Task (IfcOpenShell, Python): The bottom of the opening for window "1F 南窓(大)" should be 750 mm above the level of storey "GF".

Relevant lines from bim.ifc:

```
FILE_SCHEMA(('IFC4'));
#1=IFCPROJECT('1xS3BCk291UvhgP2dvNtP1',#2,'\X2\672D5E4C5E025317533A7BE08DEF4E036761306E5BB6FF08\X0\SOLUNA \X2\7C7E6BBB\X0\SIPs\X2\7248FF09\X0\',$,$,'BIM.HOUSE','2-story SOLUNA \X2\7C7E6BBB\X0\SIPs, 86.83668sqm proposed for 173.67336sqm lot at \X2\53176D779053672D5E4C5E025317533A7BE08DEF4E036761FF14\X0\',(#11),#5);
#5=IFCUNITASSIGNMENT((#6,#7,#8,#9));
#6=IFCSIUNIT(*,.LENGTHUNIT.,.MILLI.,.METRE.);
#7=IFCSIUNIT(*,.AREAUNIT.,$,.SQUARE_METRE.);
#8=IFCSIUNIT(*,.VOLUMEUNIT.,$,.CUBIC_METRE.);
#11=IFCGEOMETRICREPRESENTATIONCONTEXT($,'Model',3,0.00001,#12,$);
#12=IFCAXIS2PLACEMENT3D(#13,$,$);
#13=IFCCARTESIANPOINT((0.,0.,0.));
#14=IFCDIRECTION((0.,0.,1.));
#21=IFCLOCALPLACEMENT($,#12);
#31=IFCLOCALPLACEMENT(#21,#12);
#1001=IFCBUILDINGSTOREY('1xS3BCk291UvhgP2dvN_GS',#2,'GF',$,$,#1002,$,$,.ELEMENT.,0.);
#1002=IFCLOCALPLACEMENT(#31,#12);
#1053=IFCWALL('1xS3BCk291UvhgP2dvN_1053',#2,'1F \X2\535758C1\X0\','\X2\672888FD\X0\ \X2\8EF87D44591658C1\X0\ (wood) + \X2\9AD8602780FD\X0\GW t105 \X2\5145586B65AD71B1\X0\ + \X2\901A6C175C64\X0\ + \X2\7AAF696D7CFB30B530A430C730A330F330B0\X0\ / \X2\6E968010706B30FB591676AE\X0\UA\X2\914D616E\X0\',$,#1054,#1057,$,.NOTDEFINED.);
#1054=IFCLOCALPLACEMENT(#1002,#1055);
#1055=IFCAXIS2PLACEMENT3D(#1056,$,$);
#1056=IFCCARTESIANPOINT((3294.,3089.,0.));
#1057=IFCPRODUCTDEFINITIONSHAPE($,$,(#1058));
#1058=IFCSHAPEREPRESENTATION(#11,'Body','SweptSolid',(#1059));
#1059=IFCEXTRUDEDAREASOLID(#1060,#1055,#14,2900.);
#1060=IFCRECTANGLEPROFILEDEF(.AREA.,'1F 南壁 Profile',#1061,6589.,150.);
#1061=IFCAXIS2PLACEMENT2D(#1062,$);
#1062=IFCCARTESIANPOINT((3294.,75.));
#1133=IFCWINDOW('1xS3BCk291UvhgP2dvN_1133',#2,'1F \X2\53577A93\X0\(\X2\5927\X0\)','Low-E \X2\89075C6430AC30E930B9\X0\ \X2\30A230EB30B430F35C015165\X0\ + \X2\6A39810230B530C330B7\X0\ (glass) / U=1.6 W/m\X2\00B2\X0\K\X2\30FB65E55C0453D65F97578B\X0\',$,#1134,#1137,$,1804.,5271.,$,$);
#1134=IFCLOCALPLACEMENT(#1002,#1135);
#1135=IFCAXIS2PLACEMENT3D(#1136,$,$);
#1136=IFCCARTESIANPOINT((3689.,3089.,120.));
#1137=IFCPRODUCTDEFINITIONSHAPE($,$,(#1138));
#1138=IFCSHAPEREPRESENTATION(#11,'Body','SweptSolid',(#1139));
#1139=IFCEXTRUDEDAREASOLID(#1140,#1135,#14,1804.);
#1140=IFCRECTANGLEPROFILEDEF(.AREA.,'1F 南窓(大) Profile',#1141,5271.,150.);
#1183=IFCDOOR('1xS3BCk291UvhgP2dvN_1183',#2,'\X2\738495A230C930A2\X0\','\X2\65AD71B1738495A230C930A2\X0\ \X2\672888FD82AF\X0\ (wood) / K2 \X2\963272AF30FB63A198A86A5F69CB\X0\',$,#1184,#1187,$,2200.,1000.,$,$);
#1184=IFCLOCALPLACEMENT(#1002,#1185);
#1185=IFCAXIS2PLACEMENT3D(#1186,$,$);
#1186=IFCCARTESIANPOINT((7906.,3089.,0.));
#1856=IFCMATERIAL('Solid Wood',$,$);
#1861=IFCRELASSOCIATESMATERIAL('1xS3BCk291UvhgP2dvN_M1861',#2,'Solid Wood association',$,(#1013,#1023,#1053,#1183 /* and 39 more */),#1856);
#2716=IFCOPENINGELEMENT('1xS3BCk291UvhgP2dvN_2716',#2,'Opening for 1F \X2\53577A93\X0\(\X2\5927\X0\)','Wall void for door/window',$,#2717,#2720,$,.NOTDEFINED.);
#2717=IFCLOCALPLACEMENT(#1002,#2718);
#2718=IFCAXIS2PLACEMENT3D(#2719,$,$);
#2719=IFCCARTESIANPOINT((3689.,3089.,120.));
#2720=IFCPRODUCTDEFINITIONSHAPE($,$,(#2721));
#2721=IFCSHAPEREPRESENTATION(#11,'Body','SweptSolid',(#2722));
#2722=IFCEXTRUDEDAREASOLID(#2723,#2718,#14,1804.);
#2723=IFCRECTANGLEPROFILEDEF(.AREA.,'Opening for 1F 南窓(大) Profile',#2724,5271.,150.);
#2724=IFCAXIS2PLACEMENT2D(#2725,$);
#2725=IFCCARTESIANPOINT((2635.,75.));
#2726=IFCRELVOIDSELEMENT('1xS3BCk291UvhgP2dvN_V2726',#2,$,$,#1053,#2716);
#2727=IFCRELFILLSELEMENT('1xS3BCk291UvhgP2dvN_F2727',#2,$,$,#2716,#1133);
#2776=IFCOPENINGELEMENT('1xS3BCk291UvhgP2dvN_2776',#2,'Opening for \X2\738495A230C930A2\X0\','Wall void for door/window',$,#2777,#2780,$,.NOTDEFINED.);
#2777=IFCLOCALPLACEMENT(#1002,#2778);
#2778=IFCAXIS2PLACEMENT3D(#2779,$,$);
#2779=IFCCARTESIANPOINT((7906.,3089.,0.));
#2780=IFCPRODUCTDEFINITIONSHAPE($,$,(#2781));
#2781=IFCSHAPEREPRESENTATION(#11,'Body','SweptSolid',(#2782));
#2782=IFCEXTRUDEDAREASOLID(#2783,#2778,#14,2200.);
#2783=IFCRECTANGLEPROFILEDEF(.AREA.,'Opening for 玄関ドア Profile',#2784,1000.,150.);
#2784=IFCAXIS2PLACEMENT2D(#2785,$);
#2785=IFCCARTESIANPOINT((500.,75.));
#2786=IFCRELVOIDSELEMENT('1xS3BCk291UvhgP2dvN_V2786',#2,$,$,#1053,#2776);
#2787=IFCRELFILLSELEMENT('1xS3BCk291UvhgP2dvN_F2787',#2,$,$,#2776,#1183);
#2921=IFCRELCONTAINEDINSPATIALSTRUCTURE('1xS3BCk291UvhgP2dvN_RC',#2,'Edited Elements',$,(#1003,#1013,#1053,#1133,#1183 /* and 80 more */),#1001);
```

```python
import numpy as np
import ifcopenshell
import ifcopenshell.api.geometry
import ifcopenshell.geom
import ifcopenshell.util.element
import ifcopenshell.util.placement
import ifcopenshell.util.shape
import ifcopenshell.util.unit

model = ifcopenshell.open("bim.ifc")
unit_scale = ifcopenshell.util.unit.calculate_unit_scale(model)

window = model.by_id(1133)
opening = window.FillsVoids[0].RelatingOpeningElement
storey = ifcopenshell.util.element.get_container(window, ifc_class="IfcBuildingStorey")
level = ifcopenshell.util.placement.get_local_placement(storey.ObjectPlacement)[2, 3]

# The opening's origin need not be at the sill, so measure its lowest point.
shape = ifcopenshell.geom.create_shape(ifcopenshell.geom.settings(), opening)
bottom = ifcopenshell.util.shape.get_shape_bottom_elevation(shape, shape.geometry) / unit_scale
dz = level + 0.75 / unit_scale - bottom

shift = np.array([0.0, 0.0, dz])
# The window is not placed relative to its opening, so move both.
for product in (opening, window):
    matrix = ifcopenshell.util.placement.get_local_placement(product.ObjectPlacement)
    matrix[:3, 3] += shift
    ifcopenshell.api.geometry.edit_object_placement(model, product=product, matrix=matrix, is_si=False)

print(f"moved by {dz * unit_scale:+.3f} m")

model.write("bim_rev.ifc")
```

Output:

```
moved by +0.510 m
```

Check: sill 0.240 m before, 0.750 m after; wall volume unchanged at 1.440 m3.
